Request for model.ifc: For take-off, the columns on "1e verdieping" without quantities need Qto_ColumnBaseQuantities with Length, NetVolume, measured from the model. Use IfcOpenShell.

First a look at what the model holds.

```python
import ifcopenshell
import ifcopenshell.util.element
import ifcopenshell.util.unit

model = ifcopenshell.open("model.ifc")
print(model.schema)
for unit_type in ("LENGTHUNIT", "AREAUNIT", "VOLUMEUNIT"):
    print(unit_type, ifcopenshell.util.unit.calculate_unit_scale(model, unit_type))
storey = next(s for s in model.by_type("IfcBuildingStorey") if s.Name == "1e verdieping")
columns = [e for e in ifcopenshell.util.element.get_decomposition(storey) if e.is_a("IfcColumn")]
for e in sorted(columns, key=lambda e: e.id()):
    print(e.id(), e.is_a(), e.Name, list(ifcopenshell.util.element.get_psets(e, qtos_only=True)), sep=" | ")
```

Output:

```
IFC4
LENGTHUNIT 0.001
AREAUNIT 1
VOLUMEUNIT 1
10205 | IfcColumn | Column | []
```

```python
import ifcopenshell
import ifcopenshell.api.pset
import ifcopenshell.geom
import ifcopenshell.util.element
import ifcopenshell.util.shape
import ifcopenshell.util.unit

model = ifcopenshell.open("model.ifc")
unit_scale = ifcopenshell.util.unit.calculate_unit_scale(model)
volume_scale = ifcopenshell.util.unit.calculate_unit_scale(model, "VOLUMEUNIT")
settings = ifcopenshell.geom.settings()

storey = next(s for s in model.by_type("IfcBuildingStorey") if s.Name == "1e verdieping")
columns = [e for e in ifcopenshell.util.element.get_decomposition(storey) if e.is_a("IfcColumn")]

for e in sorted(columns, key=lambda e: e.id()):
    if ifcopenshell.util.element.get_psets(e, qtos_only=True, should_inherit=False):
        continue
    # Geometry comes back in metres, in the element's own axes.
    shape = ifcopenshell.geom.create_shape(settings, e)
    values = {
        "Length": ifcopenshell.util.shape.get_z(shape.geometry) / unit_scale,
        "NetVolume": ifcopenshell.util.shape.get_volume(shape.geometry) / volume_scale,
    }
    qto = ifcopenshell.api.pset.add_qto(model, product=e, name="Qto_ColumnBaseQuantities")
    ifcopenshell.api.pset.edit_qto(model, qto=qto, properties=values)
    print(e.id(), {k: round(v, 3) for k, v in values.items()})

model.write("model-out.ifc")
```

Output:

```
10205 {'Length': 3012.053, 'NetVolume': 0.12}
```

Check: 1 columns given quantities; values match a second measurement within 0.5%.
